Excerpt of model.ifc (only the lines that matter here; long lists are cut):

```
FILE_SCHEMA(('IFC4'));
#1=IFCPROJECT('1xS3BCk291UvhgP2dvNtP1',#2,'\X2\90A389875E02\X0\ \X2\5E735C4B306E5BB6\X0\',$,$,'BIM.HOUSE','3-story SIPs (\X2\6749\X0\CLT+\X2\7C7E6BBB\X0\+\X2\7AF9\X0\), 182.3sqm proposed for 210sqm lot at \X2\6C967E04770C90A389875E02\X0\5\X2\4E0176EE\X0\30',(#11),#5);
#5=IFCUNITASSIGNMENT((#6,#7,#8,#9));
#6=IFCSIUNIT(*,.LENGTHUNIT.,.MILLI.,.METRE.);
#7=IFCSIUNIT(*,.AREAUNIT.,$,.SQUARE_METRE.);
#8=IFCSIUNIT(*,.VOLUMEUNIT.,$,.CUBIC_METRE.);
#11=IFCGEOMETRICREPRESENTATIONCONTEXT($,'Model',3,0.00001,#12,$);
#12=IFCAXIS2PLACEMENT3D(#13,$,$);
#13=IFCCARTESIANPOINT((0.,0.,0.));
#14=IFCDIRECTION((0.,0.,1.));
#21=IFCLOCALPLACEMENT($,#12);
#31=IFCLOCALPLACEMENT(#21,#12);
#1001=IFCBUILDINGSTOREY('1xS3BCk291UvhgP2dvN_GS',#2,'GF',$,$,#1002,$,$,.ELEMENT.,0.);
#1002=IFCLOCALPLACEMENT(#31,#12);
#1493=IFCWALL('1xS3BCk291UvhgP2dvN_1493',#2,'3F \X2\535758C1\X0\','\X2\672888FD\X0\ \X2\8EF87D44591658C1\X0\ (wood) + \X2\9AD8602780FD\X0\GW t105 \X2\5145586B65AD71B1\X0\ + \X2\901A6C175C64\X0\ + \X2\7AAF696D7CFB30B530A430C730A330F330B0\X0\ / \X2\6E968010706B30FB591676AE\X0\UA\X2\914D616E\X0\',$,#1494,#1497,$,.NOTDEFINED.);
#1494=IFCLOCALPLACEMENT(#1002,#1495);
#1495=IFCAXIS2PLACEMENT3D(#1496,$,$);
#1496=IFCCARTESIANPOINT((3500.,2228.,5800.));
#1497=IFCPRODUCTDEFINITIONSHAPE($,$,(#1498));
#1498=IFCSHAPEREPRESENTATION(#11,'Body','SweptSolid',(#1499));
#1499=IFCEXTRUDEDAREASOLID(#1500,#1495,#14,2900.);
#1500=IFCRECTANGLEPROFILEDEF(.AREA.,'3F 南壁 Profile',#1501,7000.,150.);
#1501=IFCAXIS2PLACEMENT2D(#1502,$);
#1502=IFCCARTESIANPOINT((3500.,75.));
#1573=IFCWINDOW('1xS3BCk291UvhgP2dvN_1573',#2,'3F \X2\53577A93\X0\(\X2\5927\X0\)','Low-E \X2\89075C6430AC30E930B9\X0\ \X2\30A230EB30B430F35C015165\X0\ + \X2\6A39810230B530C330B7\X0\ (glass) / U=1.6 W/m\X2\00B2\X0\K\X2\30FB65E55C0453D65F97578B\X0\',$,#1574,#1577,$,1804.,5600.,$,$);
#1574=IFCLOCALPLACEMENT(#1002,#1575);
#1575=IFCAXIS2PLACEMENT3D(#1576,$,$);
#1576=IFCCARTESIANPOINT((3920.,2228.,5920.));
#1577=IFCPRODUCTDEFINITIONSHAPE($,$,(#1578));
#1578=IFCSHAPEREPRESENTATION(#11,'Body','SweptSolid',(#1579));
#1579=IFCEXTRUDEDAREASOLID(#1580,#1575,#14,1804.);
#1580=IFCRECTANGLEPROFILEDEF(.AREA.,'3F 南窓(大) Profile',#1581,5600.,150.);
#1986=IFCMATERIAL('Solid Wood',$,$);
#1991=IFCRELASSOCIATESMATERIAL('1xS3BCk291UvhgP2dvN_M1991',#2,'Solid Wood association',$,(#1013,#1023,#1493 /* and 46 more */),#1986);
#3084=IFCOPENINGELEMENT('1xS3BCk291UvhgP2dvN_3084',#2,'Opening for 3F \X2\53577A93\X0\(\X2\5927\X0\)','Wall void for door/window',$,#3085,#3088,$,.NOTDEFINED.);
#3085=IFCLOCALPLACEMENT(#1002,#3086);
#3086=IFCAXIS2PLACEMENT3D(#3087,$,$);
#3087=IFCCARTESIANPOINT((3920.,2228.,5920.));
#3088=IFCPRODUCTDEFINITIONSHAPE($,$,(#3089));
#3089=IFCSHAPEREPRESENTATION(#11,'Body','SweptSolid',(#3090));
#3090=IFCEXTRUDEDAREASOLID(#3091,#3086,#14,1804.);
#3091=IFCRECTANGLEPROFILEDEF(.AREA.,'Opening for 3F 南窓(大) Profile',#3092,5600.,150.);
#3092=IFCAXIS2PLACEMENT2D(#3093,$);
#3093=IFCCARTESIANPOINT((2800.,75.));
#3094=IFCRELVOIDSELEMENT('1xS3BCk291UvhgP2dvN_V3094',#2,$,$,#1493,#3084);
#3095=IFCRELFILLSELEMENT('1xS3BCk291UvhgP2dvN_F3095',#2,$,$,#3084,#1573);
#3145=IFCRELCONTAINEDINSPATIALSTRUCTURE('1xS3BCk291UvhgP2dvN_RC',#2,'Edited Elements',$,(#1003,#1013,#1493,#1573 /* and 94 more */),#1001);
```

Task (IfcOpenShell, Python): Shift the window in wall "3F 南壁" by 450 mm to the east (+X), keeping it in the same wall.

```python
import ifcopenshell
import ifcopenshell.api.geometry
import ifcopenshell.util.placement
import ifcopenshell.util.unit

model = ifcopenshell.open("model.ifc")
unit_scale = ifcopenshell.util.unit.calculate_unit_scale(model)

window = model.by_guid("1xS3BCk291UvhgP2dvN_1573")
opening = window.FillsVoids[0].RelatingOpeningElement
wall = opening.VoidsElements[0].RelatingBuildingElement

wall_matrix = ifcopenshell.util.placement.get_local_placement(wall.ObjectPlacement)
shift = wall_matrix[:3, 0] * 0.45 / unit_scale
before = ifcopenshell.util.placement.get_local_placement(window.ObjectPlacement)[:3, 3].copy()

# The window is not placed relative to its opening, so move both.
for product in (opening, window):
    matrix = ifcopenshell.util.placement.get_local_placement(product.ObjectPlacement)
    matrix[:3, 3] += shift
    ifcopenshell.api.geometry.edit_object_placement(model, product=product, matrix=matrix, is_si=False)

after = ifcopenshell.util.placement.get_local_placement(window.ObjectPlacement)[:3, 3]
print("window moved by", (after - before).round(3) + 0.0)

model.write("model_updated.ifc")
```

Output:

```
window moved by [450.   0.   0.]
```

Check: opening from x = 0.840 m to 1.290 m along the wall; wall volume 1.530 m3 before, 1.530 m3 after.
